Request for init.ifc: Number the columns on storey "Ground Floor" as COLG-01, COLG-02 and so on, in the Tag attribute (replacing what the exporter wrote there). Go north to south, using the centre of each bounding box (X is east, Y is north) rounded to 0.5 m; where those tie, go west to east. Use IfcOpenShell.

First a look at what the model holds.

```python
import ifcopenshell
import ifcopenshell.util.element
import ifcopenshell.util.placement

model = ifcopenshell.open("init.ifc")
print(model.schema)
storey = next(s for s in model.by_type("IfcBuildingStorey") if s.Name == "Ground Floor")
columns = [e for e in ifcopenshell.util.element.get_decomposition(storey) if e.is_a("IfcColumn")]
for e in sorted(columns, key=lambda e: e.id()):
    origin = ifcopenshell.util.placement.get_local_placement(e.ObjectPlacement)[:3, 3]
    print(e.id(), e.Tag, e.Name, origin.round(2) + 0.0, sep=" | ")
```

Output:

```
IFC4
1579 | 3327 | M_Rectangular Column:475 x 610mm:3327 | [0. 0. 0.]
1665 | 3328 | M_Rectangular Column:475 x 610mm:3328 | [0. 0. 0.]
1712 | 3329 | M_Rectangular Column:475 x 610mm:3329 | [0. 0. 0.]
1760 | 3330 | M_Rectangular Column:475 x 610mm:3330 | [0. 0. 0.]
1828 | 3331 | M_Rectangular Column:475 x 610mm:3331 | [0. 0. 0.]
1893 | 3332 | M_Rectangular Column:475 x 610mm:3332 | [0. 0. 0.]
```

```python
import ifcopenshell
import ifcopenshell.geom
import ifcopenshell.util.element
import ifcopenshell.util.shape

model = ifcopenshell.open("init.ifc")
settings = ifcopenshell.geom.settings()
settings.set("use-world-coords", True)


def centre(element):
    shape = ifcopenshell.geom.create_shape(settings, element)
    return ifcopenshell.util.shape.get_bbox_centroid(shape.geometry)


storey = next(s for s in model.by_type("IfcBuildingStorey") if s.Name == "Ground Floor")
columns = [e for e in ifcopenshell.util.element.get_decomposition(storey) if e.is_a("IfcColumn")]

# Insertion points can sit at a corner or the storey origin, so sort by the geometry (in metres).
centres = {e: centre(e) for e in columns}
columns.sort(key=lambda e: (-round(centres[e][1] / 0.5), centres[e][0]))

for i, e in enumerate(columns, start=1):
    number = f"COLG-{i:02d}"
    e.Tag = number
    print(e.id(), number)

model.write("init_edited.ifc")
```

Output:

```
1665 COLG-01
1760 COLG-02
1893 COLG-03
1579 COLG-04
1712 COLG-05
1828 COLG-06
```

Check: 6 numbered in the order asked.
